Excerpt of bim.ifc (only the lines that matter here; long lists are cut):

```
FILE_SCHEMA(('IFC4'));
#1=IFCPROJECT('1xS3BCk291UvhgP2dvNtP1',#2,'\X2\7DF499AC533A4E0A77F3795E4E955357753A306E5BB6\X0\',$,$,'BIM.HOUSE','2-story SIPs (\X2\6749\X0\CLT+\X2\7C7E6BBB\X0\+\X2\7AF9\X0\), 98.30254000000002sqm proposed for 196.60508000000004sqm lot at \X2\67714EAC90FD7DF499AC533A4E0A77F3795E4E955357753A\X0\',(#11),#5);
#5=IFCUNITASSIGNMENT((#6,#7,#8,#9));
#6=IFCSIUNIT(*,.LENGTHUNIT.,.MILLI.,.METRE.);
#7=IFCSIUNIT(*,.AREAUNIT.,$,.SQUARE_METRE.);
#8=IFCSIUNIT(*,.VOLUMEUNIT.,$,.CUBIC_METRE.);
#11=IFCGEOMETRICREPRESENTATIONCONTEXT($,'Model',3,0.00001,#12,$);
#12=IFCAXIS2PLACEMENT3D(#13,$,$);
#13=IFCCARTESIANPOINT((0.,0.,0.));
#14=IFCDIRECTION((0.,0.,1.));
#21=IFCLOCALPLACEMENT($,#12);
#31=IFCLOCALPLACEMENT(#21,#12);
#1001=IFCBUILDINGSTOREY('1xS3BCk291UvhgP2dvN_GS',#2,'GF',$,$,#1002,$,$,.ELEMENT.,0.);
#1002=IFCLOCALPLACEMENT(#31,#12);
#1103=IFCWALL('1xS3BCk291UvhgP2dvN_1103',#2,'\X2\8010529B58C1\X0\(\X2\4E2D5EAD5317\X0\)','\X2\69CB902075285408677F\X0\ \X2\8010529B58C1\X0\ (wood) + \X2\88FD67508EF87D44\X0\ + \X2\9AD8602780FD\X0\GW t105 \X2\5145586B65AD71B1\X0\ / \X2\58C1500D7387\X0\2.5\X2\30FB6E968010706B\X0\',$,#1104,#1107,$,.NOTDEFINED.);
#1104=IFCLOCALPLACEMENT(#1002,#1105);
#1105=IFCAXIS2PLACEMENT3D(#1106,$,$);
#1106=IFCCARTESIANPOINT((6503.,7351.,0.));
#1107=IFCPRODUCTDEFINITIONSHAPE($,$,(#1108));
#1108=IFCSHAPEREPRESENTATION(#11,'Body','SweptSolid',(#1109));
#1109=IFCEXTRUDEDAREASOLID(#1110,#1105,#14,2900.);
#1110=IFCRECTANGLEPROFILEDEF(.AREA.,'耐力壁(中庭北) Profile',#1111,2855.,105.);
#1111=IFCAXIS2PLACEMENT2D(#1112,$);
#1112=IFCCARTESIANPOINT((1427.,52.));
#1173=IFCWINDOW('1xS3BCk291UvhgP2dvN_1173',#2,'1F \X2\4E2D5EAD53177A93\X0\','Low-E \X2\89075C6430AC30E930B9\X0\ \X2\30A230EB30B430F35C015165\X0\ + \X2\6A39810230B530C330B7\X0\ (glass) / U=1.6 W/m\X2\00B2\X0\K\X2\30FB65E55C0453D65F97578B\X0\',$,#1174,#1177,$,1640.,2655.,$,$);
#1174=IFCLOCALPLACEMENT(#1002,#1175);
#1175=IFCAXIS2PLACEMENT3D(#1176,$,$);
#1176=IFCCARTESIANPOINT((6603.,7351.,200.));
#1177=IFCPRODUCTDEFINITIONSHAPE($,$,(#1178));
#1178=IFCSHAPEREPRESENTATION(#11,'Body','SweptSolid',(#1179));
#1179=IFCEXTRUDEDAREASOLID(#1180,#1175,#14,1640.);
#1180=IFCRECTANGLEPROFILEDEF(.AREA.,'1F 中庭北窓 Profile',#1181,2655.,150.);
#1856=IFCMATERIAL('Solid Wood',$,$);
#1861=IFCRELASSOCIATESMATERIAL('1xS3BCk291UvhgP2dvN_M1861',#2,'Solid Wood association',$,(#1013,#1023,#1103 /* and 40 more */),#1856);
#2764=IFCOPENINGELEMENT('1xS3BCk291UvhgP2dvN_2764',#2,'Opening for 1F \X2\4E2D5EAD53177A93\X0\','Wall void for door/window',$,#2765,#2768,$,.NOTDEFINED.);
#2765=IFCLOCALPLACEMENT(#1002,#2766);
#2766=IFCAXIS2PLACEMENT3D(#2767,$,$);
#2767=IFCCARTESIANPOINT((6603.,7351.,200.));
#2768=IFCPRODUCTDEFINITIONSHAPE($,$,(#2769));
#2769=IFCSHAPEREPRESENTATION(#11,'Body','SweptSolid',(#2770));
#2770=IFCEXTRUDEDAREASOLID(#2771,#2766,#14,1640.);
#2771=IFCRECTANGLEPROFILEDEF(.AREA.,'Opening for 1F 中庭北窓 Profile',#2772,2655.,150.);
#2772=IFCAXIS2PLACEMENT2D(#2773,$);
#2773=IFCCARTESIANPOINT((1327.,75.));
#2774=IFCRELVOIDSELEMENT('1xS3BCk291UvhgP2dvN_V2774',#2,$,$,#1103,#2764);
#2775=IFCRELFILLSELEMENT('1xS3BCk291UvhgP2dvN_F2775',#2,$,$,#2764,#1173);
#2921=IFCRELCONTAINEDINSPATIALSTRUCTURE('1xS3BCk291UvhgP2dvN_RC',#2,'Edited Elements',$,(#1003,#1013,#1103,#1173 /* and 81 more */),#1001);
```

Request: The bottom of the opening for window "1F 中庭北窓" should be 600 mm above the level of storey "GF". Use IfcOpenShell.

```python
import numpy as np
import ifcopenshell
import ifcopenshell.api.geometry
import ifcopenshell.geom
import ifcopenshell.util.element
import ifcopenshell.util.placement
import ifcopenshell.util.shape
import ifcopenshell.util.unit

model = ifcopenshell.open("bim.ifc")
unit_scale = ifcopenshell.util.unit.calculate_unit_scale(model)

window = model.by_guid("1xS3BCk291UvhgP2dvN_1173")
opening = window.FillsVoids[0].RelatingOpeningElement
storey = ifcopenshell.util.element.get_container(window, ifc_class="IfcBuildingStorey")
level = ifcopenshell.util.placement.get_local_placement(storey.ObjectPlacement)[2, 3]

# The opening's origin need not be at the sill, so measure its lowest point.
shape = ifcopenshell.geom.create_shape(ifcopenshell.geom.settings(), opening)
bottom = ifcopenshell.util.shape.get_shape_bottom_elevation(shape, shape.geometry) / unit_scale
dz = level + 600.0 - bottom

shift = np.array([0.0, 0.0, dz])
# The window is not placed relative to its opening, so move both.
for product in (opening, window):
    matrix = ifcopenshell.util.placement.get_local_placement(product.ObjectPlacement)
    matrix[:3, 3] += shift
    ifcopenshell.api.geometry.edit_object_placement(model, product=product, matrix=matrix, is_si=False)

print(f"moved by {dz * unit_scale:+.3f} m")

model.write("bim-out.ifc")
```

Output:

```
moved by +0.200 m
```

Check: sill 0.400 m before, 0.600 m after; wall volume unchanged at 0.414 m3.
